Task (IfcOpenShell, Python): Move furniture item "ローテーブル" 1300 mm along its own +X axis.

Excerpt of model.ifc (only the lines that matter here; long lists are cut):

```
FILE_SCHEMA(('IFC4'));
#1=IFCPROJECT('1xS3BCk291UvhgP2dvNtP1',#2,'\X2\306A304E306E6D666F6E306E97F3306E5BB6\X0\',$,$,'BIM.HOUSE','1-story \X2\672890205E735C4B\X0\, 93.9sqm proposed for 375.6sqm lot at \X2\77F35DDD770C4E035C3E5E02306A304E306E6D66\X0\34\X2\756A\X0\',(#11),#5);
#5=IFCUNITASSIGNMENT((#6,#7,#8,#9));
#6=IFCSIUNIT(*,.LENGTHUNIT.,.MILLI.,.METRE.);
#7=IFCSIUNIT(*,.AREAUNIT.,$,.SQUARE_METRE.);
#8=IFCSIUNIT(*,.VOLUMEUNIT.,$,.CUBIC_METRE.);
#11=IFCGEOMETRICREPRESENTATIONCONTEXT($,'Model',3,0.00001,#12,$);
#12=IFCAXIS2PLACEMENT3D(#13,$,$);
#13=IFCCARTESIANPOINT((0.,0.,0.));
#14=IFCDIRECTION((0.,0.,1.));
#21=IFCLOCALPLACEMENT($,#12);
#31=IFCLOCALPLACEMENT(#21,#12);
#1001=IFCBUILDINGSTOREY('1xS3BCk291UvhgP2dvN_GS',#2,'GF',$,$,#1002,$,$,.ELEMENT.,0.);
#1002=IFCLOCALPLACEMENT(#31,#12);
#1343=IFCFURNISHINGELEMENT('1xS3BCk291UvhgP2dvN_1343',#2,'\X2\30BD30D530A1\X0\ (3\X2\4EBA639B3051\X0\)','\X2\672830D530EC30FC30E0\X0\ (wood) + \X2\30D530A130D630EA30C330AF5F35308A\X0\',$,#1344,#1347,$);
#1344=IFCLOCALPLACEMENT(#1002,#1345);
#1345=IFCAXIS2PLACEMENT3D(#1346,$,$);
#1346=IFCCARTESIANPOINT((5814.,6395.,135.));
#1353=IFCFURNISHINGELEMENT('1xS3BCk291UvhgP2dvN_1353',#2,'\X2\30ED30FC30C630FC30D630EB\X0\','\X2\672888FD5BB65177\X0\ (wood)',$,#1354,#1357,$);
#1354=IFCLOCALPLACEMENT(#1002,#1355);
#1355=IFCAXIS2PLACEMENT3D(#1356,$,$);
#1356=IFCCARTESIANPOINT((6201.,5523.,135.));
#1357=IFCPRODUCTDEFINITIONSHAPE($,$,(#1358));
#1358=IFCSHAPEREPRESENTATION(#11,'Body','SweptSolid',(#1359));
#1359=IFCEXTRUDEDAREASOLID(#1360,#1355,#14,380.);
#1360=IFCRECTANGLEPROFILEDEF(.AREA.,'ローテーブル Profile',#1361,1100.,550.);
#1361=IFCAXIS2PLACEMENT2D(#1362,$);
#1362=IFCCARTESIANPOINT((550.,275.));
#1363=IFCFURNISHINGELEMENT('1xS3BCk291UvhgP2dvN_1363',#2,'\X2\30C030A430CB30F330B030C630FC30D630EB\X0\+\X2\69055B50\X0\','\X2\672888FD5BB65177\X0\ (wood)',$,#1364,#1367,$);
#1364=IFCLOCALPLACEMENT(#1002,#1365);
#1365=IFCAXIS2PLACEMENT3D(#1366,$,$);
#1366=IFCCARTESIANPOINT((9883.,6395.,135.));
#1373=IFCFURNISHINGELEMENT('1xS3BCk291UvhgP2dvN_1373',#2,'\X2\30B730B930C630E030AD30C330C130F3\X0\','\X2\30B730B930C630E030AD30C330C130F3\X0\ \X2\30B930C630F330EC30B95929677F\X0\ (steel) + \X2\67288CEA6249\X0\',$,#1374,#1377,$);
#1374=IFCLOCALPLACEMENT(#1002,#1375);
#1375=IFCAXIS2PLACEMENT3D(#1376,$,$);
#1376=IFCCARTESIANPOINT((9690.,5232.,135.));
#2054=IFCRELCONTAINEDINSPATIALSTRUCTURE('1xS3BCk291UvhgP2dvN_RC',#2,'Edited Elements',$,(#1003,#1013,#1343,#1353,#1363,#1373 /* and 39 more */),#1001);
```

```python
import ifcopenshell
import ifcopenshell.api.geometry
import ifcopenshell.util.placement
import ifcopenshell.util.unit

model = ifcopenshell.open("model.ifc")
unit_scale = ifcopenshell.util.unit.calculate_unit_scale(model)

item = model.by_guid("1xS3BCk291UvhgP2dvN_1353")
matrix = ifcopenshell.util.placement.get_local_placement(item.ObjectPlacement)
matrix[:3, 3] += matrix[:3, 0] * 1.3 / unit_scale
ifcopenshell.api.geometry.edit_object_placement(model, product=item, matrix=matrix, is_si=False)

print(ifcopenshell.util.placement.get_local_placement(item.ObjectPlacement).round(3) + 0.0)

model.write("model_edited.ifc")
```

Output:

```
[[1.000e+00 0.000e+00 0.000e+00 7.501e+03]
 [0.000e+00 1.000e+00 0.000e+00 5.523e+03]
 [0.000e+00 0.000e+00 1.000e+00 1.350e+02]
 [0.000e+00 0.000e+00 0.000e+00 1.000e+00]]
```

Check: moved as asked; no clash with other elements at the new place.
